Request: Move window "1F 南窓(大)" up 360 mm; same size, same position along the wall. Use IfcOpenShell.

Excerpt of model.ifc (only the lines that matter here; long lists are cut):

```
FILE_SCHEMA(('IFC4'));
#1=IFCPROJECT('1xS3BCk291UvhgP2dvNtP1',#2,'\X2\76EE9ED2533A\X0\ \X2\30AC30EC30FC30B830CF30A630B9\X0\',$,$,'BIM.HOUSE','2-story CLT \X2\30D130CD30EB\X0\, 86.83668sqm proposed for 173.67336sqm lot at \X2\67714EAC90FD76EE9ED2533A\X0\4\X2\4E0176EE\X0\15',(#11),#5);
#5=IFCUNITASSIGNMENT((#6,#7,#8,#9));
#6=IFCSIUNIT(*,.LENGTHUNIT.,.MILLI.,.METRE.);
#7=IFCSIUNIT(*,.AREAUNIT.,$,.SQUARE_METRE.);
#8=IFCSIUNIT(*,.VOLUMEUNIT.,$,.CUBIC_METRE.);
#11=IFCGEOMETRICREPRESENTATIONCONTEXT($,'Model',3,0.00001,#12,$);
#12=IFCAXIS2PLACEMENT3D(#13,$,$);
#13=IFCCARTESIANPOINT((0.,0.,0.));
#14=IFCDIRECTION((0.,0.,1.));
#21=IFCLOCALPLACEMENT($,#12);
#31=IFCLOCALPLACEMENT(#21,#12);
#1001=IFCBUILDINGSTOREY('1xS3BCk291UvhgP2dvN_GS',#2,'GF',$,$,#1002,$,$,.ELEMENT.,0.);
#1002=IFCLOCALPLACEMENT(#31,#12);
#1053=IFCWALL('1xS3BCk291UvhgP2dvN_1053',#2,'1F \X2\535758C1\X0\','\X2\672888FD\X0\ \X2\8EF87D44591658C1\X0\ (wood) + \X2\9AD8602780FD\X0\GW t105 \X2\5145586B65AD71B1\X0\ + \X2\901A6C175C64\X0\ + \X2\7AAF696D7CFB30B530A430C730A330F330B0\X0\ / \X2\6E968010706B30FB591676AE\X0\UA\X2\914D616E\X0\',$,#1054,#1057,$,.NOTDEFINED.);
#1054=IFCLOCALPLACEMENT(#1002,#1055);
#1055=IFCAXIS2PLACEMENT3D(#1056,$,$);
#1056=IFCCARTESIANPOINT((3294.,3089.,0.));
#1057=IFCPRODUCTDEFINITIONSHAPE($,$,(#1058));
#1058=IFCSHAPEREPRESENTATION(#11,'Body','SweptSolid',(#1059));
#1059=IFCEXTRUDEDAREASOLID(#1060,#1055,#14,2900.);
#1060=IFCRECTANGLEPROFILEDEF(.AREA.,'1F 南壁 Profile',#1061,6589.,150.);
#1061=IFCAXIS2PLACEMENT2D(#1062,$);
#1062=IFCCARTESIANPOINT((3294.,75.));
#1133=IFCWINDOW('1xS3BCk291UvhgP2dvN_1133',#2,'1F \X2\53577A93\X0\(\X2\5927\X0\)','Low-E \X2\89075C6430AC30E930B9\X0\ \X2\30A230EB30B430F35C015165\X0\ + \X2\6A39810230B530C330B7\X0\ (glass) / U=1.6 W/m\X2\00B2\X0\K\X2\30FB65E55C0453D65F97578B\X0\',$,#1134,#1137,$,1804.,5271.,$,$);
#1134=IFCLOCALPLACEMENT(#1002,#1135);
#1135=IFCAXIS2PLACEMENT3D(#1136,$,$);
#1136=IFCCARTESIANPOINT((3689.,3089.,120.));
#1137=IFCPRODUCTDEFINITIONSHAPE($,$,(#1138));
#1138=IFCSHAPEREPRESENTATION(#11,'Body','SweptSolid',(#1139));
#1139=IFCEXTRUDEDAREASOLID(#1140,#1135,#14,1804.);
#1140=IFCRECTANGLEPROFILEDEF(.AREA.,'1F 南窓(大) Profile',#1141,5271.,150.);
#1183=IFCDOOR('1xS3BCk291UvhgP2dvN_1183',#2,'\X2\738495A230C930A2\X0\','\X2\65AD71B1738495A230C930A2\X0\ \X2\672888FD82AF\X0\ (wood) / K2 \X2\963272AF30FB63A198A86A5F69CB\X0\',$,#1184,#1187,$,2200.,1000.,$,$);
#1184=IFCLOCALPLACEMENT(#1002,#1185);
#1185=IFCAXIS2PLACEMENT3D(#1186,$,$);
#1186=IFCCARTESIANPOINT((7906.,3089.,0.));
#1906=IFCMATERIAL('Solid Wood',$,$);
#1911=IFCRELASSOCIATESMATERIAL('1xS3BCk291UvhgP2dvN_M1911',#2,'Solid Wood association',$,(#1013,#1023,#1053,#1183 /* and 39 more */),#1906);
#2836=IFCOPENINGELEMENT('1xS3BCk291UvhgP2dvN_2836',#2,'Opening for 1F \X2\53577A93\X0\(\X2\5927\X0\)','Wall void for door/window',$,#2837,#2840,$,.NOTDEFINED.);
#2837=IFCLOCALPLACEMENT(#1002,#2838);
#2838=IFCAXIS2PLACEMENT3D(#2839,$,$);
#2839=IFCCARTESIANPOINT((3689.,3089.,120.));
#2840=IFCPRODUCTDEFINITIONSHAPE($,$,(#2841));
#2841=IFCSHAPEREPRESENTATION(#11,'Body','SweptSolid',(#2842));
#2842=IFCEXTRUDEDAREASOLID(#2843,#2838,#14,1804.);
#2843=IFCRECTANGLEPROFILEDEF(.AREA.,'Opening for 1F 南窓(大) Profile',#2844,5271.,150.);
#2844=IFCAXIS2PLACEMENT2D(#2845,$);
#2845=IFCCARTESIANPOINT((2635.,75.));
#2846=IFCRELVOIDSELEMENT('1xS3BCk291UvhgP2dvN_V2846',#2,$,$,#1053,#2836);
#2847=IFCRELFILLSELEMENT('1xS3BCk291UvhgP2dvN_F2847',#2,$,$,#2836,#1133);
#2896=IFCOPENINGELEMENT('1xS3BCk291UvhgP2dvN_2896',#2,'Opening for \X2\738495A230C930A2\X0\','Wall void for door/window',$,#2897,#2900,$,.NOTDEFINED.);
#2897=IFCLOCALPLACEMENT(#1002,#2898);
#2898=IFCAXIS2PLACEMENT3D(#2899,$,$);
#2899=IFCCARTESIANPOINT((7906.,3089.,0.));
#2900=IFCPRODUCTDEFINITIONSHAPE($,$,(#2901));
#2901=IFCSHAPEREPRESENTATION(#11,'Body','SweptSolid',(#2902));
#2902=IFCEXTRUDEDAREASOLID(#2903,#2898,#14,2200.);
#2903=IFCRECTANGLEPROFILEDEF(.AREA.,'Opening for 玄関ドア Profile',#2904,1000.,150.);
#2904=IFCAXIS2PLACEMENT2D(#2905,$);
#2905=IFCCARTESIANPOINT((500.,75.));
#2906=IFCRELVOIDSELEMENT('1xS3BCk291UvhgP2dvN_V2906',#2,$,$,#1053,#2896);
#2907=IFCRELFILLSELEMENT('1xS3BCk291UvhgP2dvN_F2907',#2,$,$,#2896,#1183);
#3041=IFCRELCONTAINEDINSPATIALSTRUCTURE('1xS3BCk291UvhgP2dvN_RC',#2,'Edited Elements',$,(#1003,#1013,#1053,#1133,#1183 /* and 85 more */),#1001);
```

```python
import numpy as np
import ifcopenshell
import ifcopenshell.api.geometry
import ifcopenshell.util.placement
import ifcopenshell.util.unit

model = ifcopenshell.open("model.ifc")
unit_scale = ifcopenshell.util.unit.calculate_unit_scale(model)

window = model.by_guid("1xS3BCk291UvhgP2dvN_1133")
opening = window.FillsVoids[0].RelatingOpeningElement
dz = 360.0

shift = np.array([0.0, 0.0, dz])
# The window is not placed relative to its opening, so move both.
for product in (opening, window):
    matrix = ifcopenshell.util.placement.get_local_placement(product.ObjectPlacement)
    matrix[:3, 3] += shift
    ifcopenshell.api.geometry.edit_object_placement(model, product=product, matrix=matrix, is_si=False)

print(f"moved by {dz * unit_scale:+.3f} m")

model.write("model-out.ifc")
```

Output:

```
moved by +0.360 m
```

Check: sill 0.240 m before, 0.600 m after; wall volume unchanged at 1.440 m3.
